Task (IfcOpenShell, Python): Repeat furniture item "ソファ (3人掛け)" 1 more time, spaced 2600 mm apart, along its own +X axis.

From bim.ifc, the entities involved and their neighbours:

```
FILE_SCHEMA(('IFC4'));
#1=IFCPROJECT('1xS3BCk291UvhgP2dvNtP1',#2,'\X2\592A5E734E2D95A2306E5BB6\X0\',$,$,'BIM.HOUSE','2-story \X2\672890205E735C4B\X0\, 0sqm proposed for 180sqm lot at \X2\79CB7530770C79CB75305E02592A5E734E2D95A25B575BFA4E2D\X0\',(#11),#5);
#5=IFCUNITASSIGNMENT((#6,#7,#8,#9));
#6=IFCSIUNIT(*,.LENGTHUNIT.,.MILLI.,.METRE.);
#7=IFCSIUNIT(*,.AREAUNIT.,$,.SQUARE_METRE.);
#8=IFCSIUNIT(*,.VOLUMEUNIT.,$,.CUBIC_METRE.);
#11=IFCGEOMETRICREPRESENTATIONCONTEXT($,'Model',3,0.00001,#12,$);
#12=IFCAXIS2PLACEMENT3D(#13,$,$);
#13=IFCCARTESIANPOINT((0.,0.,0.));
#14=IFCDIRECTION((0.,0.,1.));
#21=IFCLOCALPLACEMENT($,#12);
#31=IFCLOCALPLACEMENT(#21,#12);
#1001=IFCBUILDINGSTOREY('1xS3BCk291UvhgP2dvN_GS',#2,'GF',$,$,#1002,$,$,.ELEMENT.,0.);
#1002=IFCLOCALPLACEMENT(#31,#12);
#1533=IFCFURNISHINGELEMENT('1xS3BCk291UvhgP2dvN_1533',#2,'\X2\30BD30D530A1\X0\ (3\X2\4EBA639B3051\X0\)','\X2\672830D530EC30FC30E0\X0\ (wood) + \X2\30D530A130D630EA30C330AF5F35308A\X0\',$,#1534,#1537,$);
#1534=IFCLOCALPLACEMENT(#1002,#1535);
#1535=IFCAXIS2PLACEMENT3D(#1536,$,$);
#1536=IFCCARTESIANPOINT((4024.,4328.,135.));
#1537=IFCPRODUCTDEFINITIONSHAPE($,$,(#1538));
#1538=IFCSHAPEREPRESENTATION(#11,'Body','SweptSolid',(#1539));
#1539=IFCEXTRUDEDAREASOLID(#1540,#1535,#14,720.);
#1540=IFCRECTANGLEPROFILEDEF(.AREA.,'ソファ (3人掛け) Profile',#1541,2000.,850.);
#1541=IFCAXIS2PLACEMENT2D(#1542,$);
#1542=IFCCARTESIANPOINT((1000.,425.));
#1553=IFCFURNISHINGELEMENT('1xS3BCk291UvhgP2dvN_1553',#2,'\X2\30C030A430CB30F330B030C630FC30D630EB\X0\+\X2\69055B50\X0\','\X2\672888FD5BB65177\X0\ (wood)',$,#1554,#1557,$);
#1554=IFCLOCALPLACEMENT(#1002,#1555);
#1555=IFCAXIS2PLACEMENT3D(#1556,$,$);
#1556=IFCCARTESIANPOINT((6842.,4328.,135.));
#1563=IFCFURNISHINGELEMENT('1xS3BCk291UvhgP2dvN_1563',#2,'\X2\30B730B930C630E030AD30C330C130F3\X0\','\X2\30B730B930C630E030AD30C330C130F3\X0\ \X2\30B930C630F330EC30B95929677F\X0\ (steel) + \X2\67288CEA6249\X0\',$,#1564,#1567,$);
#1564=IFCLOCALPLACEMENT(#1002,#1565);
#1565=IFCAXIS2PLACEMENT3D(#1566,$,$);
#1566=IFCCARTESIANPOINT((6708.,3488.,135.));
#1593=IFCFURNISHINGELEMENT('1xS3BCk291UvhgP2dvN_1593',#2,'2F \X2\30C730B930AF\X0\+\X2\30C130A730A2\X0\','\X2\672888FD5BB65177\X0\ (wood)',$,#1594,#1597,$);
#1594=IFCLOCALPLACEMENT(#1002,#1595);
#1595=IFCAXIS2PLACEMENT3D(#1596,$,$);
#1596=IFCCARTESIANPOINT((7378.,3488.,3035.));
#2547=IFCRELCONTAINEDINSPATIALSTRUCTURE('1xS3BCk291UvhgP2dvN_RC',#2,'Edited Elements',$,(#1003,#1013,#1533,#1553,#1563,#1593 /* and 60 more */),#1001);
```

```python
import ifcopenshell
import ifcopenshell.api.geometry
import ifcopenshell.api.root
import ifcopenshell.util.element
import ifcopenshell.util.placement
import ifcopenshell.util.unit

model = ifcopenshell.open("bim.ifc")
unit_scale = ifcopenshell.util.unit.calculate_unit_scale(model)


def reuse_history(source, copy):
    """copy_class also copies each property set's owner history, people and application; keep the originals."""
    for rel in copy.IsDefinedBy:
        if rel.is_a("IfcRelDefinesByProperties") and (history := rel.RelatingPropertyDefinition.OwnerHistory):
            rel.RelatingPropertyDefinition.OwnerHistory = source.OwnerHistory
            ifcopenshell.util.element.remove_deep2(model, history)


source = model.by_guid("1xS3BCk291UvhgP2dvN_1533")
base = ifcopenshell.util.placement.get_local_placement(source.ObjectPlacement)
step = base[:3, 0] * 2.6 / unit_scale

for i in range(1, 2):
    copy = ifcopenshell.api.root.copy_class(model, product=source)
    copy.Representation = ifcopenshell.util.element.copy_deep(
        model, source.Representation, exclude=["IfcGeometricRepresentationContext", "IfcRepresentationMap"]
    )
    reuse_history(source, copy)
    matrix = base.copy()
    matrix[:3, 3] += i * step
    print("added at", matrix[:3, 3].round(3) + 0.0)
    ifcopenshell.api.geometry.edit_object_placement(model, product=copy, matrix=matrix, is_si=False)

model.write("bim_updated.ifc")
```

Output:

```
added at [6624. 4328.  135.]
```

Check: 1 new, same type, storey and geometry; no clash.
